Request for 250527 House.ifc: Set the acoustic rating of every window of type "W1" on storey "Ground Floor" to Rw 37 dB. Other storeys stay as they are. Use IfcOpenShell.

First a look at what the model holds.

```python
import ifcopenshell
import ifcopenshell.util.element

model = ifcopenshell.open("250527 House.ifc")
print(model.schema)
storey = next(s for s in model.by_type("IfcBuildingStorey") if s.Name == "Ground Floor")
windows = [e for e in ifcopenshell.util.element.get_decomposition(storey) if e.is_a("IfcWindow")]
seen = {}
for e in windows:
    element_type = ifcopenshell.util.element.get_type(e)
    key = (element_type.Name if element_type != e and element_type else None, ifcopenshell.util.element.get_pset(e, "Pset_WindowCommon", "AcousticRating"))
    seen[key] = seen.get(key, 0) + 1
for (name, value), count in sorted(seen.items(), key=str):
    print(count, "x", name, "|", value)
```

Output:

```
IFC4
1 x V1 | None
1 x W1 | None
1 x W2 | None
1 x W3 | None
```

```python
import ifcopenshell
import ifcopenshell.api.pset
import ifcopenshell.util.element

model = ifcopenshell.open("250527 House.ifc")

storey = next(s for s in model.by_type("IfcBuildingStorey") if s.Name == "Ground Floor")
windows = [e for e in ifcopenshell.util.element.get_decomposition(storey) if e.is_a("IfcWindow")]

count = 0
for e in windows:
    element_type = ifcopenshell.util.element.get_type(e)
    if element_type in (None, e) or element_type.Name != "W1":
        continue
    # add_pset returns the element's existing set when there is one.
    pset = ifcopenshell.api.pset.add_pset(model, product=e, name="Pset_WindowCommon")
    ifcopenshell.api.pset.edit_pset(model, pset=pset, properties={"AcousticRating": "Rw 37 dB"})
    count += 1

print(count, "windows updated")

model.write("250527 House_v2.ifc")
```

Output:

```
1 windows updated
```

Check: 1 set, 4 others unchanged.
